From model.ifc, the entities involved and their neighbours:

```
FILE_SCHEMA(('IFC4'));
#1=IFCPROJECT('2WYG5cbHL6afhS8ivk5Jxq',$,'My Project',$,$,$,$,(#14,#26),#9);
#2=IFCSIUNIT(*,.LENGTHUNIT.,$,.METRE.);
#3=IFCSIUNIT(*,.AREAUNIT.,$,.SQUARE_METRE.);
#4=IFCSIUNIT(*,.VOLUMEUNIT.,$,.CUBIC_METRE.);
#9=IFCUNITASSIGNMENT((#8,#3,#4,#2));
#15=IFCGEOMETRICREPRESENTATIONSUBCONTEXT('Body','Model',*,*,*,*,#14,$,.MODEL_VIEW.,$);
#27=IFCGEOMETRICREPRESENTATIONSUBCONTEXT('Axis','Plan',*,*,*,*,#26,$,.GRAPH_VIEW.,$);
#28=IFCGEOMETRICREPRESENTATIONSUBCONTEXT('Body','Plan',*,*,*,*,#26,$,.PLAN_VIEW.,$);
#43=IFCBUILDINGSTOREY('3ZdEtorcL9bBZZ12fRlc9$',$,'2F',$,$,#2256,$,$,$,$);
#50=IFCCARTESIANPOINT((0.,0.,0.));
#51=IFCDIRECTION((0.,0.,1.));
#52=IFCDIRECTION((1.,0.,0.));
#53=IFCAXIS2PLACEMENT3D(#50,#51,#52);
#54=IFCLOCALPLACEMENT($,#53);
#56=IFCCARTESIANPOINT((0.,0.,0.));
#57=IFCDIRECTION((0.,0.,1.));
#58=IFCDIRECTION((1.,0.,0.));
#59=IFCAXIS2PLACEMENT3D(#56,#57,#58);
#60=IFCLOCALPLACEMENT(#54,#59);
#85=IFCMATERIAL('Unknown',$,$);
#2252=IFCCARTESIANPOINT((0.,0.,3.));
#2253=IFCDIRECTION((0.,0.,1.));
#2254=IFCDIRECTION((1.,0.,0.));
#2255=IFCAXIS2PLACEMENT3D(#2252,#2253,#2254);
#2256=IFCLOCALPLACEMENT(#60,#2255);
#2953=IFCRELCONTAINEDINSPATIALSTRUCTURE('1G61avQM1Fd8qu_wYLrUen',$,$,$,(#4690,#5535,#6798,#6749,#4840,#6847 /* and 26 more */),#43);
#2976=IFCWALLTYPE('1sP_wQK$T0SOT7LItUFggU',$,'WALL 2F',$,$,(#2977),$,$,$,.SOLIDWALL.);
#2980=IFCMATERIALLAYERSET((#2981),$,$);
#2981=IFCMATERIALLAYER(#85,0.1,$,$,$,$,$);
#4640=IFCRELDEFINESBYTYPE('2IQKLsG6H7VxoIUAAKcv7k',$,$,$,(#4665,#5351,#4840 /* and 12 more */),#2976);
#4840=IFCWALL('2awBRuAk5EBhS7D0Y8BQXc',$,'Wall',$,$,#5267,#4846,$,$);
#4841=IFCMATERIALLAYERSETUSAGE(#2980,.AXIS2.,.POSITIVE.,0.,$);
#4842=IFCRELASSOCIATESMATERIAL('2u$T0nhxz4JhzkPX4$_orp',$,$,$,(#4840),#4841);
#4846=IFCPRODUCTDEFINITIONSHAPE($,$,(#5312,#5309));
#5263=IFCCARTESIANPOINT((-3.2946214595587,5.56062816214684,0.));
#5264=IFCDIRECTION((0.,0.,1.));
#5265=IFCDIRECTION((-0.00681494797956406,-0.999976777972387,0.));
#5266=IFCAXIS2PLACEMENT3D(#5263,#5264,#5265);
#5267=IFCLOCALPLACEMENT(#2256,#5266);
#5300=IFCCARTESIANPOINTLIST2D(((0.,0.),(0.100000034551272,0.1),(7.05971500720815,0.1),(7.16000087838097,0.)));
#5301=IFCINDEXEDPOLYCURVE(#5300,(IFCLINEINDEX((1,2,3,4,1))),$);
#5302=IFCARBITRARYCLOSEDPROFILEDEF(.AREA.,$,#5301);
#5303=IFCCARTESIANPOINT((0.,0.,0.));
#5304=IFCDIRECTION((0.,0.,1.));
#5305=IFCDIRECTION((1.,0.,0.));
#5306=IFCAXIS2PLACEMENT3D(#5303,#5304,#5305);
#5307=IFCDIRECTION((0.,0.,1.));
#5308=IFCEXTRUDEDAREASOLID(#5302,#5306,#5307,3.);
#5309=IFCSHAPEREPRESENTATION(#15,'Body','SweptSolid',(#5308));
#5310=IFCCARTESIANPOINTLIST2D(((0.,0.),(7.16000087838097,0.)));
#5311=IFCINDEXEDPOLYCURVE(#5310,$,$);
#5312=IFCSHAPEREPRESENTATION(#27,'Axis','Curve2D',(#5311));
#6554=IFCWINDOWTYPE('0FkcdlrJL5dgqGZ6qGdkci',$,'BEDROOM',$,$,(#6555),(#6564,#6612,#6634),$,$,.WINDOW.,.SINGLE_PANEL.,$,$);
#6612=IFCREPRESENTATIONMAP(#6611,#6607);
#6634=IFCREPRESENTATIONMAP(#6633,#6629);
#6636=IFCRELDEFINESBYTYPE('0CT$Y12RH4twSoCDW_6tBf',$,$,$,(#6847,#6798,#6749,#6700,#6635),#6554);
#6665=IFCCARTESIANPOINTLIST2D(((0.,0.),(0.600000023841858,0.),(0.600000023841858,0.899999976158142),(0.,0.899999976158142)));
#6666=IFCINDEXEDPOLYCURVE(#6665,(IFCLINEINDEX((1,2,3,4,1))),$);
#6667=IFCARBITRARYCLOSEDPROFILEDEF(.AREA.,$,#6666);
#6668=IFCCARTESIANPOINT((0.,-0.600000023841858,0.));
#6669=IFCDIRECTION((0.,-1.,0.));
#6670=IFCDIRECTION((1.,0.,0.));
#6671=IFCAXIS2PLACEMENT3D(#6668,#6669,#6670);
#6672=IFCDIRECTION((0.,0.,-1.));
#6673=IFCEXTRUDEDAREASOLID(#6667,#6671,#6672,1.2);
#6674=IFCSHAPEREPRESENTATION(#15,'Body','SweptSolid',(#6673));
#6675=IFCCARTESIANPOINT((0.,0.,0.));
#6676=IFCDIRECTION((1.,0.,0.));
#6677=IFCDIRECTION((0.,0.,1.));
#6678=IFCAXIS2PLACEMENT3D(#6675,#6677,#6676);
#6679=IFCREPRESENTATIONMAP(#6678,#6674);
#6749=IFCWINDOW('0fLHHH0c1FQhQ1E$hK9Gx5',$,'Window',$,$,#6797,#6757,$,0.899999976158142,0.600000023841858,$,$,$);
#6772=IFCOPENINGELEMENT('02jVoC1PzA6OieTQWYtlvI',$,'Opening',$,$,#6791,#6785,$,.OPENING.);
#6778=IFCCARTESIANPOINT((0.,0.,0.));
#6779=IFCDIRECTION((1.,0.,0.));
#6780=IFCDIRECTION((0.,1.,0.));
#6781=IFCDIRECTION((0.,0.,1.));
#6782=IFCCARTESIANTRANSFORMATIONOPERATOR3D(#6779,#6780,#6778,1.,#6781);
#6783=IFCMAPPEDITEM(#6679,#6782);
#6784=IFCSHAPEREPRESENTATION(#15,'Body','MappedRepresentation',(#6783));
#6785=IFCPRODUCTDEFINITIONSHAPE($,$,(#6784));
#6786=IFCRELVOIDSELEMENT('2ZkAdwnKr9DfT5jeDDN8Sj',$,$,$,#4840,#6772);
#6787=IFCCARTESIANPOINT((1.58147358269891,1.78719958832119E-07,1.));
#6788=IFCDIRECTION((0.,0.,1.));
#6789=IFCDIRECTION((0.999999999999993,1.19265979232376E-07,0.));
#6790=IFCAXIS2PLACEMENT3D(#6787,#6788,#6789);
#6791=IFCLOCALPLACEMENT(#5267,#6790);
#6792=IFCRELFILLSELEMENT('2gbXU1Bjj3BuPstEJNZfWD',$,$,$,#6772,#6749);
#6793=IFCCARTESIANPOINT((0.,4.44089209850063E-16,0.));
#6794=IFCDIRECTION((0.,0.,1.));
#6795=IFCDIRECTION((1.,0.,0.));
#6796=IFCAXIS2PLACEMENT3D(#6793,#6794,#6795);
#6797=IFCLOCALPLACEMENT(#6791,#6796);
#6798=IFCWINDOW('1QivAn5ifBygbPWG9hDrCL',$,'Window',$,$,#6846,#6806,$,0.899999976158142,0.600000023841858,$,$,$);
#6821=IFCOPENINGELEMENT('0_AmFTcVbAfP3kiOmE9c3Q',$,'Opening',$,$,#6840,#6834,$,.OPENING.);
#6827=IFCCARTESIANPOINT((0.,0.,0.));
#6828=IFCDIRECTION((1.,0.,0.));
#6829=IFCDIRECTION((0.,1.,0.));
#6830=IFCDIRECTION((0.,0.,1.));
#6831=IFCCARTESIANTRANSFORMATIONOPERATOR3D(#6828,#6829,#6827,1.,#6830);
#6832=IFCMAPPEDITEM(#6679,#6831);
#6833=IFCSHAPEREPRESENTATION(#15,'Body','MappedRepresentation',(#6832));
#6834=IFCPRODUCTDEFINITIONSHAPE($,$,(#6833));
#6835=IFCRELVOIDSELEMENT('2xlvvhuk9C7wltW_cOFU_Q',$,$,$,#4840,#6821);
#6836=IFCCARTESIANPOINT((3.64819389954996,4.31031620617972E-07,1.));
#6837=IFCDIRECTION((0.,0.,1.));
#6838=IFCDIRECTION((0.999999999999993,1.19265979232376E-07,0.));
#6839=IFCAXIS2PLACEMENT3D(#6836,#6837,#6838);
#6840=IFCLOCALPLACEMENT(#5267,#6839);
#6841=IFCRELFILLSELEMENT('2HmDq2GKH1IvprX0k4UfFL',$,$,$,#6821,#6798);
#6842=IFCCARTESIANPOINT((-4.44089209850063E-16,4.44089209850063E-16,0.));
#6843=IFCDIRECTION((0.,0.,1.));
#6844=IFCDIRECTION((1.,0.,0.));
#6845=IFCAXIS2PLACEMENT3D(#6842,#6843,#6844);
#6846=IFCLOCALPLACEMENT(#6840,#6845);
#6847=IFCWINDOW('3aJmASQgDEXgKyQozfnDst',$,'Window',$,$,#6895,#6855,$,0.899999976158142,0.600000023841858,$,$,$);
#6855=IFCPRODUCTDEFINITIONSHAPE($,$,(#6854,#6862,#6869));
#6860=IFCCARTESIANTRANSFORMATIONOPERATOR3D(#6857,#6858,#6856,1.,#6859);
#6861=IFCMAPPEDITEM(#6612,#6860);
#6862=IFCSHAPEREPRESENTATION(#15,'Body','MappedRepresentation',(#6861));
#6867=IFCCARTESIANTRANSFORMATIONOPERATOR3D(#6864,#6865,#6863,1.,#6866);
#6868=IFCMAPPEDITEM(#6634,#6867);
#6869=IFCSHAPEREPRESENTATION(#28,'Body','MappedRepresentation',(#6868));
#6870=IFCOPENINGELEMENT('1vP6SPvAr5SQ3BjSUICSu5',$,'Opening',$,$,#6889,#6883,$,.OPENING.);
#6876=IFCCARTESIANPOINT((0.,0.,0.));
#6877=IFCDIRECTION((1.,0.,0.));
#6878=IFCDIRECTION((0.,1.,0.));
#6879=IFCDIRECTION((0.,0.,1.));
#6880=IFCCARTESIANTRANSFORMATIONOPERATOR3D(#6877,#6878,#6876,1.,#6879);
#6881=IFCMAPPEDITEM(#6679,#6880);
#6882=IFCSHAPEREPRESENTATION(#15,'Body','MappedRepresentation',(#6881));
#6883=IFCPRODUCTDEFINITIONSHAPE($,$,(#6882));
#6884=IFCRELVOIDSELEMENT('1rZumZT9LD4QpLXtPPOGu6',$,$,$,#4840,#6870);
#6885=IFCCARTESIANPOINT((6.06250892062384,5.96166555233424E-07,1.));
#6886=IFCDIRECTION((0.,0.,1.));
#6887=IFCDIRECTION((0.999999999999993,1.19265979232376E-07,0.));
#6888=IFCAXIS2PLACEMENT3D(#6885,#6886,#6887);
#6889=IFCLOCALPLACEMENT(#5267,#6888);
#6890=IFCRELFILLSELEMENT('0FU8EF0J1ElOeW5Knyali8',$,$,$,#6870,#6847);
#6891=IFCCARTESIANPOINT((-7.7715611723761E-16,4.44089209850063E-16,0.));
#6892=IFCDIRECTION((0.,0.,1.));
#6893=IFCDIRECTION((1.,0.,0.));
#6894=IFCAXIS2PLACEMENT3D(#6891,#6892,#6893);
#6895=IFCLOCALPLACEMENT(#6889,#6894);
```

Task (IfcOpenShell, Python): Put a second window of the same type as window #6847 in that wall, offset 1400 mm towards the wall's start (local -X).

```python
import ifcopenshell
import ifcopenshell.api.feature
import ifcopenshell.api.geometry
import ifcopenshell.api.root
import ifcopenshell.geom
import ifcopenshell.util.element
import ifcopenshell.util.placement
import ifcopenshell.util.shape
import ifcopenshell.util.unit

model = ifcopenshell.open("model.ifc")
unit_scale = ifcopenshell.util.unit.calculate_unit_scale(model)
settings = ifcopenshell.geom.settings()


def volume(element):
    """Net volume in cubic metres, openings subtracted."""
    shape = ifcopenshell.geom.create_shape(settings, element)
    return ifcopenshell.util.shape.get_volume(shape.geometry)


window = model.by_guid("3aJmASQgDEXgKyQozfnDst")
opening = window.FillsVoids[0].RelatingOpeningElement
wall = opening.VoidsElements[0].RelatingBuildingElement
before = volume(wall)
shift = ifcopenshell.util.placement.get_local_placement(wall.ObjectPlacement)[:3, 0] * -1.4 / unit_scale

# copy_class copies the void relationship, type, container and properties, but no geometry.
new_opening = ifcopenshell.api.root.copy_class(model, product=opening)
new_opening.Representation = ifcopenshell.util.element.copy_deep(
    model, opening.Representation, exclude=["IfcGeometricRepresentationContext", "IfcRepresentationMap"]
)
new_window = ifcopenshell.api.root.copy_class(model, product=window)
new_window.Representation = ifcopenshell.util.element.copy_deep(
    model, window.Representation, exclude=["IfcGeometricRepresentationContext", "IfcRepresentationMap"]
)
ifcopenshell.api.feature.add_filling(model, opening=new_opening, element=new_window)

for old, new in ((opening, new_opening), (window, new_window)):
    matrix = ifcopenshell.util.placement.get_local_placement(old.ObjectPlacement)
    matrix[:3, 3] += shift
    ifcopenshell.api.geometry.edit_object_placement(model, product=new, matrix=matrix, is_si=False)

after = volume(wall)

print(f"wall volume {before:.3f} -> {after:.3f} m3")

model.write("model_updated.ifc")
```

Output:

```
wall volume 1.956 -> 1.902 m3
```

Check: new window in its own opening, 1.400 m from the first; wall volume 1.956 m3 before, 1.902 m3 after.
